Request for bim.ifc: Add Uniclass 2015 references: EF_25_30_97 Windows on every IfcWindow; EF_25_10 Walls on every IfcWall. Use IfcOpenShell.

First a look at what the model holds.

```python
import ifcopenshell

model = ifcopenshell.open("bim.ifc")
print(model.schema)
print("classifications:", [c.Name for c in model.by_type("IfcClassification")])
for ifc_class in ("IfcDoor", "IfcRoof", "IfcStair", "IfcWall", "IfcWindow"):
    print(ifc_class, len(model.by_type(ifc_class)))
```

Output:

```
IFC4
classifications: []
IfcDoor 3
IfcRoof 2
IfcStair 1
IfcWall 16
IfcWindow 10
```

```python
import ifcopenshell
import ifcopenshell.api.classification

model = ifcopenshell.open("bim.ifc")

system = ifcopenshell.api.classification.add_classification(model, classification="Uniclass 2015")

codes = {
    "IfcWindow": ("EF_25_30_97", "Windows"),
    "IfcWall": ("EF_25_10", "Walls"),
}
for ifc_class, (code, name) in codes.items():
    products = model.by_type(ifc_class)
    ifcopenshell.api.classification.add_reference(
        model, products=products, classification=system, identification=code, name=name
    )
    print(code, len(products))

model.write("bim-out.ifc")
```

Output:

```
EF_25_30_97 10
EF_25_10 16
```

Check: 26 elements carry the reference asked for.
